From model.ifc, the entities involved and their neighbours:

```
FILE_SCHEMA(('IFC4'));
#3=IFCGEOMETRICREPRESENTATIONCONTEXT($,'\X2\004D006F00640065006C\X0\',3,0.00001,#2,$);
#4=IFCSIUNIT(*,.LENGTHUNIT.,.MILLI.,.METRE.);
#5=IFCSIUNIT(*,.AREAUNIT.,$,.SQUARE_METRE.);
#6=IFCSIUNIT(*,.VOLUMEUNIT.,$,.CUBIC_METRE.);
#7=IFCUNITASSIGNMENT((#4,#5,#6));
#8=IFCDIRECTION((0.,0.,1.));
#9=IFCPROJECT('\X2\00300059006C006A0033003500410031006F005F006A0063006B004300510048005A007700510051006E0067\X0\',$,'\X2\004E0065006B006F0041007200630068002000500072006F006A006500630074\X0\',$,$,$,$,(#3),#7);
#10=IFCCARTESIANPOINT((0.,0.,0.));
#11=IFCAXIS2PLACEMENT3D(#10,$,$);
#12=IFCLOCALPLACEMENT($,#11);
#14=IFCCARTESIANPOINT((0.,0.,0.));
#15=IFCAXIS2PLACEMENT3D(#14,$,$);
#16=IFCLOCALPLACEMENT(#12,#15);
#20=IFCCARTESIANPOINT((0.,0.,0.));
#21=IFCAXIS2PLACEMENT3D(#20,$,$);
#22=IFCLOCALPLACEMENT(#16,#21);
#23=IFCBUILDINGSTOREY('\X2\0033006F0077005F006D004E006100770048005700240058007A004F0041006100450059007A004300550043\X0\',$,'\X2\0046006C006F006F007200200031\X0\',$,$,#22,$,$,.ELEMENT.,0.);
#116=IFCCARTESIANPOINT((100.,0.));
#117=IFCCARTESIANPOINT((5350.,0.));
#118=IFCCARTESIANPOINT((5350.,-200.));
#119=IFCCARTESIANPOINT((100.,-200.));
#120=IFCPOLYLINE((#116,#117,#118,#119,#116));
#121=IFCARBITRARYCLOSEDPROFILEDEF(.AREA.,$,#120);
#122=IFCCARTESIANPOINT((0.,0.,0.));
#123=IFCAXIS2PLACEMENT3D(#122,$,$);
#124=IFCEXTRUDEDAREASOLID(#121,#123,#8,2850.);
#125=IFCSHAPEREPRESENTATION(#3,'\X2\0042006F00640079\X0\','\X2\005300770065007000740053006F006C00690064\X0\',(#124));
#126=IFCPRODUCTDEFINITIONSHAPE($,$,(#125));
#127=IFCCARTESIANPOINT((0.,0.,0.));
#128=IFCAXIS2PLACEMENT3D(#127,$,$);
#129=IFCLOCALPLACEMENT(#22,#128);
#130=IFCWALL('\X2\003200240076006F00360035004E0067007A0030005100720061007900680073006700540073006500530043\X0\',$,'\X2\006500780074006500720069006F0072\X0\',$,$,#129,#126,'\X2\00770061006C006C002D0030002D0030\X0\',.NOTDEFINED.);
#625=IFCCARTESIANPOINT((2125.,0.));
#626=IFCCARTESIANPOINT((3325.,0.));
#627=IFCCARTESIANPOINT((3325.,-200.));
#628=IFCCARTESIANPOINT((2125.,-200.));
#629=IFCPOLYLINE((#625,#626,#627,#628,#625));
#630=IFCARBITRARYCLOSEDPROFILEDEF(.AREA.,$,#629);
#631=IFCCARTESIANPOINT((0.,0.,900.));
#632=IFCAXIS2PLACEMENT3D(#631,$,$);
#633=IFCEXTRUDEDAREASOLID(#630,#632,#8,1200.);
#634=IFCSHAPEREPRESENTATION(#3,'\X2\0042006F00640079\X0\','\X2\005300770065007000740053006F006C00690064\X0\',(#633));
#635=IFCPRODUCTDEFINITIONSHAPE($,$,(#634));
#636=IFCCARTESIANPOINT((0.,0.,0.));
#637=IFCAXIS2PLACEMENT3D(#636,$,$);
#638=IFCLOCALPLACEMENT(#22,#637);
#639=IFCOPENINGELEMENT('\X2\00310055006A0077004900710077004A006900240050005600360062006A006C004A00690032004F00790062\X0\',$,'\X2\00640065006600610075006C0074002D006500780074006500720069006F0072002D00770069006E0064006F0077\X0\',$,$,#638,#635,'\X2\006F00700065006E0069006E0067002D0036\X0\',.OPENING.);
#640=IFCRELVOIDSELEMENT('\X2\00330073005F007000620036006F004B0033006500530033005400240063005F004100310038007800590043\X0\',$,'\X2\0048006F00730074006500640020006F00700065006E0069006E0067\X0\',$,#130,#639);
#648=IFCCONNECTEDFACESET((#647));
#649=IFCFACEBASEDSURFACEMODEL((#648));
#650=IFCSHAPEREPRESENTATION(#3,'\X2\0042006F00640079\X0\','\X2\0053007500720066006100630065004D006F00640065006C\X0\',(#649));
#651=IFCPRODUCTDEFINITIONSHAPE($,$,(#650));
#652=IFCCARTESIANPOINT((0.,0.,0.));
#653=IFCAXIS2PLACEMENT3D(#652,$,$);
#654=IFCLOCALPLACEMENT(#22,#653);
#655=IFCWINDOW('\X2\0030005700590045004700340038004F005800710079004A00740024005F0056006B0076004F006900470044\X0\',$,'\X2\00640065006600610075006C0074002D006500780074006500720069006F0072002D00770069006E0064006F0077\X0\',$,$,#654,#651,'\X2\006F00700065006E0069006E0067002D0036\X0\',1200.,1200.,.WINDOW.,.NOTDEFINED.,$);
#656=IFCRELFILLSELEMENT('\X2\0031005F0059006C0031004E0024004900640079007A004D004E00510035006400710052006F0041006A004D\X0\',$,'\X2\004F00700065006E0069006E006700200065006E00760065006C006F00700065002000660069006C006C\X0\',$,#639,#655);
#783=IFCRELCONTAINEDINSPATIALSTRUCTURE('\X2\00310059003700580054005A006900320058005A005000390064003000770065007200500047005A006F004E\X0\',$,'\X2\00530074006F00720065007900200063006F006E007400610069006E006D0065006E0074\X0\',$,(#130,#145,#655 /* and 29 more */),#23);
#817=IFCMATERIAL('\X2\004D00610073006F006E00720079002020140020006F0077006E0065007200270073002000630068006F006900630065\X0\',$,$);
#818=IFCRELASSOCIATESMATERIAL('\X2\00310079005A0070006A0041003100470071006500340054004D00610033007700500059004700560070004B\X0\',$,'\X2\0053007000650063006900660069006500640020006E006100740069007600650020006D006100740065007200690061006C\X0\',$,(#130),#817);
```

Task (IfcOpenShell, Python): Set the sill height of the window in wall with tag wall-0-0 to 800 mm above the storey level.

```python
import numpy as np
import ifcopenshell
import ifcopenshell.api.geometry
import ifcopenshell.geom
import ifcopenshell.util.element
import ifcopenshell.util.placement
import ifcopenshell.util.shape
import ifcopenshell.util.unit

model = ifcopenshell.open("model.ifc")
unit_scale = ifcopenshell.util.unit.calculate_unit_scale(model)

window = model.by_guid("0WYEG48OXqyJt$_VkvOiGD")
opening = window.FillsVoids[0].RelatingOpeningElement
storey = ifcopenshell.util.element.get_container(window, ifc_class="IfcBuildingStorey")
level = ifcopenshell.util.placement.get_local_placement(storey.ObjectPlacement)[2, 3]

# The opening's origin need not be at the sill, so measure its lowest point.
shape = ifcopenshell.geom.create_shape(ifcopenshell.geom.settings(), opening)
bottom = ifcopenshell.util.shape.get_shape_bottom_elevation(shape, shape.geometry) / unit_scale
dz = level + 800.0 - bottom

shift = np.array([0.0, 0.0, dz])
# The window is not placed relative to its opening, so move both.
for product in (opening, window):
    matrix = ifcopenshell.util.placement.get_local_placement(product.ObjectPlacement)
    matrix[:3, 3] += shift
    ifcopenshell.api.geometry.edit_object_placement(model, product=product, matrix=matrix, is_si=False)

print(f"moved by {dz * unit_scale:+.3f} m")

model.write("model_v2.ifc")
```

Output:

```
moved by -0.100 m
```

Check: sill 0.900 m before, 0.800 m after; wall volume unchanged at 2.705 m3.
